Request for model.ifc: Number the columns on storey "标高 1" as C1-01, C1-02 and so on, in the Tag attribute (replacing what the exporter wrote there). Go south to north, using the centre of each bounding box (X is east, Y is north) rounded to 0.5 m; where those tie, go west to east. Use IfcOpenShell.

First a look at what the model holds.

```python
import ifcopenshell
import ifcopenshell.util.element
import ifcopenshell.util.placement

model = ifcopenshell.open("model.ifc")
print(model.schema)
storey = next(s for s in model.by_type("IfcBuildingStorey") if s.Name == "标高 1")
columns = [e for e in ifcopenshell.util.element.get_decomposition(storey) if e.is_a("IfcColumn")]
for e in sorted(columns, key=lambda e: e.id()):
    origin = ifcopenshell.util.placement.get_local_placement(e.ObjectPlacement)[:3, 3]
    print(e.id(), e.Tag, e.Name, origin.round(2) + 0.0, sep=" | ")
```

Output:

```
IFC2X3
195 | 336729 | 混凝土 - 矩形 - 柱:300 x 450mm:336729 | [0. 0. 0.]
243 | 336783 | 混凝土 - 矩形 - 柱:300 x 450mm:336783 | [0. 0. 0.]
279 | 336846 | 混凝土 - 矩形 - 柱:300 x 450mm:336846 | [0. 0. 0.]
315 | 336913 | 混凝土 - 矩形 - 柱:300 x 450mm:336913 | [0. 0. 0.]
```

```python
import ifcopenshell
import ifcopenshell.geom
import ifcopenshell.util.element
import ifcopenshell.util.shape

model = ifcopenshell.open("model.ifc")
settings = ifcopenshell.geom.settings()
settings.set("use-world-coords", True)


def centre(element):
    shape = ifcopenshell.geom.create_shape(settings, element)
    return ifcopenshell.util.shape.get_bbox_centroid(shape.geometry)


storey = next(s for s in model.by_type("IfcBuildingStorey") if s.Name == "标高 1")
columns = [e for e in ifcopenshell.util.element.get_decomposition(storey) if e.is_a("IfcColumn")]

# Insertion points can sit at a corner or the storey origin, so sort by the geometry (in metres).
centres = {e: centre(e) for e in columns}
columns.sort(key=lambda e: (round(centres[e][1] / 0.5), centres[e][0]))

for i, e in enumerate(columns, start=1):
    number = f"C1-{i:02d}"
    e.Tag = number
    print(e.id(), number)

model.write("model-out.ifc")
```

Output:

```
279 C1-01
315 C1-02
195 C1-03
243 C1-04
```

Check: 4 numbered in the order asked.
